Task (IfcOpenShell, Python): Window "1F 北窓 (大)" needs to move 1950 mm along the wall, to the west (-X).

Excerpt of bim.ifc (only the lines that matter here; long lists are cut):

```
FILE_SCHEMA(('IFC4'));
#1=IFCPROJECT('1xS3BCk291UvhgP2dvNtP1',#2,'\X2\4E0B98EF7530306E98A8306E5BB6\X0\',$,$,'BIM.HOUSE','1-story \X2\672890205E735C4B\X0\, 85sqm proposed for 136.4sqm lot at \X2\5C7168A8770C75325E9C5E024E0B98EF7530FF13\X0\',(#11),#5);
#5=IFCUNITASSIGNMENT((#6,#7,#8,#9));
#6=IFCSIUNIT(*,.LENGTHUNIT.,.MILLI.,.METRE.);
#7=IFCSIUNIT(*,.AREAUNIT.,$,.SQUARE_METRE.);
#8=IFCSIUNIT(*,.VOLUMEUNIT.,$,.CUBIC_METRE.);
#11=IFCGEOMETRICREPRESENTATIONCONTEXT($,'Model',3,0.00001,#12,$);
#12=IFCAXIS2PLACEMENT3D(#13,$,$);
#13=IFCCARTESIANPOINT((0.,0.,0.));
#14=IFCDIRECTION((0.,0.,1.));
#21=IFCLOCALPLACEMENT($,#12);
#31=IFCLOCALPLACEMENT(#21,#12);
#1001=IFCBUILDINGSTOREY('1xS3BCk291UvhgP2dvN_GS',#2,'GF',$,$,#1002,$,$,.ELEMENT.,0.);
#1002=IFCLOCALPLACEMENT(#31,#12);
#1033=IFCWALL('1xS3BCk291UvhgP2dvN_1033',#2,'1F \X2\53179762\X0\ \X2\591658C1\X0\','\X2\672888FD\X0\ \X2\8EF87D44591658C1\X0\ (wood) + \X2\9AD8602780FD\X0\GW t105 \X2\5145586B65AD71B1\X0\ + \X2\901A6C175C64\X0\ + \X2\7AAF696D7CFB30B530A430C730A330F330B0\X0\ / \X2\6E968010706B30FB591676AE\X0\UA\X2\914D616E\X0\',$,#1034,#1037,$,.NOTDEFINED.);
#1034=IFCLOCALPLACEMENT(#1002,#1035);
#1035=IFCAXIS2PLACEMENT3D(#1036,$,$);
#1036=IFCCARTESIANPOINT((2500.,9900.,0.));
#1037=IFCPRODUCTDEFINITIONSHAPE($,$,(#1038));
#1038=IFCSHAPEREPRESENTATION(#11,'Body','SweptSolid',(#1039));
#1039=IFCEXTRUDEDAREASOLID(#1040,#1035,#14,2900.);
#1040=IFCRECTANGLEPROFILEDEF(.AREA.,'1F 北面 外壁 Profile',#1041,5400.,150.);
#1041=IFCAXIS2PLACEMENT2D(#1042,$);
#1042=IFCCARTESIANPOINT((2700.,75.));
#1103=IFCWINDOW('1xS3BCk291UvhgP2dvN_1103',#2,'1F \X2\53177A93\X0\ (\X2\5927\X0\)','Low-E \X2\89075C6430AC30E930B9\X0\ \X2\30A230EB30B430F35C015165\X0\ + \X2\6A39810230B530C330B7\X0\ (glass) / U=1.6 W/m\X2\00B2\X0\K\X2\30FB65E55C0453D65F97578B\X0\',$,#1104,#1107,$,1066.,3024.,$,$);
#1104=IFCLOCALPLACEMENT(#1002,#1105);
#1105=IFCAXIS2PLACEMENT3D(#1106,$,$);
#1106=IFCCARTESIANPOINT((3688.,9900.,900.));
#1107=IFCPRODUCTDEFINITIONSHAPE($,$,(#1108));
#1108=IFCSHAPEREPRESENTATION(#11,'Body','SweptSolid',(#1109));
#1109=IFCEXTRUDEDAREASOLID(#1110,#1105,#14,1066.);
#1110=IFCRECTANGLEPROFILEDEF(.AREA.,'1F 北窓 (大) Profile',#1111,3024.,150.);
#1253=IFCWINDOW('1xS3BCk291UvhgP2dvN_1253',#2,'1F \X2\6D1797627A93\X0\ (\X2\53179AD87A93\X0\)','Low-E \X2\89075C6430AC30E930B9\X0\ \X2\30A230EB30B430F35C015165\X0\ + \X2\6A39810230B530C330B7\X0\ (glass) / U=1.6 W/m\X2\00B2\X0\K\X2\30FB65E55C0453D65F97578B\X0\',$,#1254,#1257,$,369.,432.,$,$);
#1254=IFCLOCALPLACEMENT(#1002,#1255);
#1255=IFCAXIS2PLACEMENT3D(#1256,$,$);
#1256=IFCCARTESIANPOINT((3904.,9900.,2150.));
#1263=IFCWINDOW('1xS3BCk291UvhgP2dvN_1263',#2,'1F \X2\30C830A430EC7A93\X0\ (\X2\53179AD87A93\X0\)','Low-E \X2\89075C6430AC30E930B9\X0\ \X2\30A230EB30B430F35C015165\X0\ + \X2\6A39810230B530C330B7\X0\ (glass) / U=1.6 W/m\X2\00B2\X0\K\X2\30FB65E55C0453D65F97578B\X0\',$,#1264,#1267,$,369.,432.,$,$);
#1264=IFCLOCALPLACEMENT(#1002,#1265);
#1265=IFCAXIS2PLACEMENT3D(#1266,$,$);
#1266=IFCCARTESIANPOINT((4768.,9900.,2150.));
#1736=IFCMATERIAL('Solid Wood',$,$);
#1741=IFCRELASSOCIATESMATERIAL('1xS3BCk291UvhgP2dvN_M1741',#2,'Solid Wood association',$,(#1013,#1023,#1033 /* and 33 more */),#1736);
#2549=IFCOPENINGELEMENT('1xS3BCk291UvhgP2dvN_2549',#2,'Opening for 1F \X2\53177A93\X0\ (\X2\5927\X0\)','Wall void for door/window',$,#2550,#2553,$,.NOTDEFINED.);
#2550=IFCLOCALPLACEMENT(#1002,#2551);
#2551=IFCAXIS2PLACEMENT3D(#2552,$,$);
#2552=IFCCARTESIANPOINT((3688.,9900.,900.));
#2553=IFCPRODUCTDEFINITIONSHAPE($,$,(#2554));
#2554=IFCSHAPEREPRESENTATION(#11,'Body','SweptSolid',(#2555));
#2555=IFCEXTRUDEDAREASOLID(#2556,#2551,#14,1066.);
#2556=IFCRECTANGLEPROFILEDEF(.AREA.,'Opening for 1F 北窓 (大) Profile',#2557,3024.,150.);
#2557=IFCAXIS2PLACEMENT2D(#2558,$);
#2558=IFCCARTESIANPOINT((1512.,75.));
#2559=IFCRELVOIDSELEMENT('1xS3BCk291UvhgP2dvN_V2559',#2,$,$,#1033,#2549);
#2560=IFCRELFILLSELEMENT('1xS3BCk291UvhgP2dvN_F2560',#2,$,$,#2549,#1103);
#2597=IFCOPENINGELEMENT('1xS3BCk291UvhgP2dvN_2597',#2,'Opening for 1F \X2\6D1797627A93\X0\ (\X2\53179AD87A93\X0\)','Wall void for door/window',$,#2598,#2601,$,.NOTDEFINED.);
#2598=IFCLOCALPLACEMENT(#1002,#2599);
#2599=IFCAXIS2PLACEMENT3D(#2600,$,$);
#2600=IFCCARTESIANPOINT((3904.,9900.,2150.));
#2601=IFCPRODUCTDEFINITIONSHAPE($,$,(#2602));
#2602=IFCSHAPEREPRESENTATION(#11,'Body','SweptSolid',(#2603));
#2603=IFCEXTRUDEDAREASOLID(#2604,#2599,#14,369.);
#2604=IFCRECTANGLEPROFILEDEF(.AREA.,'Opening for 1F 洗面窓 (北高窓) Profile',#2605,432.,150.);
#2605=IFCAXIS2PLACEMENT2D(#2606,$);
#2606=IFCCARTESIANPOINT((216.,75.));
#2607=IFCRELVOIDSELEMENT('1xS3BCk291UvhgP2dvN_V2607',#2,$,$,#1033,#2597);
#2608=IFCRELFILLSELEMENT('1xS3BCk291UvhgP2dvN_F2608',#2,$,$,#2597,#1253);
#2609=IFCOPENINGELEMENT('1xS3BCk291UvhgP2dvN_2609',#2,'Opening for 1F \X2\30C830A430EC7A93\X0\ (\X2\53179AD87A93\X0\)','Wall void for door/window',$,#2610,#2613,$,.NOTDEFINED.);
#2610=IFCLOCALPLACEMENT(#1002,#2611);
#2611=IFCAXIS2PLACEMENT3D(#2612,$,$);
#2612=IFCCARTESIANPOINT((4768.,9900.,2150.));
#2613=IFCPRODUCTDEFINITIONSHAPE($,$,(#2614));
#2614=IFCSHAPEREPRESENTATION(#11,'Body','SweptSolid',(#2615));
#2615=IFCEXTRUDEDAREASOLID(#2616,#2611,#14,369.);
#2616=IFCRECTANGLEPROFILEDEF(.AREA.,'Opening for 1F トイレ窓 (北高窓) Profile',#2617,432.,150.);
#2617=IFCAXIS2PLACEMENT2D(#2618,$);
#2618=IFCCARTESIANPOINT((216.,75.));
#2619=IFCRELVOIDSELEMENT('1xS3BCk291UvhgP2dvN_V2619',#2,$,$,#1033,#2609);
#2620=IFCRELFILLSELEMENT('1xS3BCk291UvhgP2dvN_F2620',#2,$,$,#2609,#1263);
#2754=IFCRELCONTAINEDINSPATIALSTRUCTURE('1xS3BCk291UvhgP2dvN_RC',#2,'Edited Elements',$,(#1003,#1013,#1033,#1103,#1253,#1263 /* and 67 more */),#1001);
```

```python
import ifcopenshell
import ifcopenshell.api.geometry
import ifcopenshell.util.placement

model = ifcopenshell.open("bim.ifc")

window = model.by_guid("1xS3BCk291UvhgP2dvN_1103")
opening = window.FillsVoids[0].RelatingOpeningElement
wall = opening.VoidsElements[0].RelatingBuildingElement

wall_matrix = ifcopenshell.util.placement.get_local_placement(wall.ObjectPlacement)
shift = wall_matrix[:3, 0] * -1950.0
before = ifcopenshell.util.placement.get_local_placement(window.ObjectPlacement)[:3, 3].copy()

# The window is not placed relative to its opening, so move both.
for product in (opening, window):
    matrix = ifcopenshell.util.placement.get_local_placement(product.ObjectPlacement)
    matrix[:3, 3] += shift
    ifcopenshell.api.geometry.edit_object_placement(model, product=product, matrix=matrix, is_si=False)

after = ifcopenshell.util.placement.get_local_placement(window.ObjectPlacement)[:3, 3]
print("window moved by", (after - before).round(3) + 0.0)

model.write("bim_updated.ifc")
```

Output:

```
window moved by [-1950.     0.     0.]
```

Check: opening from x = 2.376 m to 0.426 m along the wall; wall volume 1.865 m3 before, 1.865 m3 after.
